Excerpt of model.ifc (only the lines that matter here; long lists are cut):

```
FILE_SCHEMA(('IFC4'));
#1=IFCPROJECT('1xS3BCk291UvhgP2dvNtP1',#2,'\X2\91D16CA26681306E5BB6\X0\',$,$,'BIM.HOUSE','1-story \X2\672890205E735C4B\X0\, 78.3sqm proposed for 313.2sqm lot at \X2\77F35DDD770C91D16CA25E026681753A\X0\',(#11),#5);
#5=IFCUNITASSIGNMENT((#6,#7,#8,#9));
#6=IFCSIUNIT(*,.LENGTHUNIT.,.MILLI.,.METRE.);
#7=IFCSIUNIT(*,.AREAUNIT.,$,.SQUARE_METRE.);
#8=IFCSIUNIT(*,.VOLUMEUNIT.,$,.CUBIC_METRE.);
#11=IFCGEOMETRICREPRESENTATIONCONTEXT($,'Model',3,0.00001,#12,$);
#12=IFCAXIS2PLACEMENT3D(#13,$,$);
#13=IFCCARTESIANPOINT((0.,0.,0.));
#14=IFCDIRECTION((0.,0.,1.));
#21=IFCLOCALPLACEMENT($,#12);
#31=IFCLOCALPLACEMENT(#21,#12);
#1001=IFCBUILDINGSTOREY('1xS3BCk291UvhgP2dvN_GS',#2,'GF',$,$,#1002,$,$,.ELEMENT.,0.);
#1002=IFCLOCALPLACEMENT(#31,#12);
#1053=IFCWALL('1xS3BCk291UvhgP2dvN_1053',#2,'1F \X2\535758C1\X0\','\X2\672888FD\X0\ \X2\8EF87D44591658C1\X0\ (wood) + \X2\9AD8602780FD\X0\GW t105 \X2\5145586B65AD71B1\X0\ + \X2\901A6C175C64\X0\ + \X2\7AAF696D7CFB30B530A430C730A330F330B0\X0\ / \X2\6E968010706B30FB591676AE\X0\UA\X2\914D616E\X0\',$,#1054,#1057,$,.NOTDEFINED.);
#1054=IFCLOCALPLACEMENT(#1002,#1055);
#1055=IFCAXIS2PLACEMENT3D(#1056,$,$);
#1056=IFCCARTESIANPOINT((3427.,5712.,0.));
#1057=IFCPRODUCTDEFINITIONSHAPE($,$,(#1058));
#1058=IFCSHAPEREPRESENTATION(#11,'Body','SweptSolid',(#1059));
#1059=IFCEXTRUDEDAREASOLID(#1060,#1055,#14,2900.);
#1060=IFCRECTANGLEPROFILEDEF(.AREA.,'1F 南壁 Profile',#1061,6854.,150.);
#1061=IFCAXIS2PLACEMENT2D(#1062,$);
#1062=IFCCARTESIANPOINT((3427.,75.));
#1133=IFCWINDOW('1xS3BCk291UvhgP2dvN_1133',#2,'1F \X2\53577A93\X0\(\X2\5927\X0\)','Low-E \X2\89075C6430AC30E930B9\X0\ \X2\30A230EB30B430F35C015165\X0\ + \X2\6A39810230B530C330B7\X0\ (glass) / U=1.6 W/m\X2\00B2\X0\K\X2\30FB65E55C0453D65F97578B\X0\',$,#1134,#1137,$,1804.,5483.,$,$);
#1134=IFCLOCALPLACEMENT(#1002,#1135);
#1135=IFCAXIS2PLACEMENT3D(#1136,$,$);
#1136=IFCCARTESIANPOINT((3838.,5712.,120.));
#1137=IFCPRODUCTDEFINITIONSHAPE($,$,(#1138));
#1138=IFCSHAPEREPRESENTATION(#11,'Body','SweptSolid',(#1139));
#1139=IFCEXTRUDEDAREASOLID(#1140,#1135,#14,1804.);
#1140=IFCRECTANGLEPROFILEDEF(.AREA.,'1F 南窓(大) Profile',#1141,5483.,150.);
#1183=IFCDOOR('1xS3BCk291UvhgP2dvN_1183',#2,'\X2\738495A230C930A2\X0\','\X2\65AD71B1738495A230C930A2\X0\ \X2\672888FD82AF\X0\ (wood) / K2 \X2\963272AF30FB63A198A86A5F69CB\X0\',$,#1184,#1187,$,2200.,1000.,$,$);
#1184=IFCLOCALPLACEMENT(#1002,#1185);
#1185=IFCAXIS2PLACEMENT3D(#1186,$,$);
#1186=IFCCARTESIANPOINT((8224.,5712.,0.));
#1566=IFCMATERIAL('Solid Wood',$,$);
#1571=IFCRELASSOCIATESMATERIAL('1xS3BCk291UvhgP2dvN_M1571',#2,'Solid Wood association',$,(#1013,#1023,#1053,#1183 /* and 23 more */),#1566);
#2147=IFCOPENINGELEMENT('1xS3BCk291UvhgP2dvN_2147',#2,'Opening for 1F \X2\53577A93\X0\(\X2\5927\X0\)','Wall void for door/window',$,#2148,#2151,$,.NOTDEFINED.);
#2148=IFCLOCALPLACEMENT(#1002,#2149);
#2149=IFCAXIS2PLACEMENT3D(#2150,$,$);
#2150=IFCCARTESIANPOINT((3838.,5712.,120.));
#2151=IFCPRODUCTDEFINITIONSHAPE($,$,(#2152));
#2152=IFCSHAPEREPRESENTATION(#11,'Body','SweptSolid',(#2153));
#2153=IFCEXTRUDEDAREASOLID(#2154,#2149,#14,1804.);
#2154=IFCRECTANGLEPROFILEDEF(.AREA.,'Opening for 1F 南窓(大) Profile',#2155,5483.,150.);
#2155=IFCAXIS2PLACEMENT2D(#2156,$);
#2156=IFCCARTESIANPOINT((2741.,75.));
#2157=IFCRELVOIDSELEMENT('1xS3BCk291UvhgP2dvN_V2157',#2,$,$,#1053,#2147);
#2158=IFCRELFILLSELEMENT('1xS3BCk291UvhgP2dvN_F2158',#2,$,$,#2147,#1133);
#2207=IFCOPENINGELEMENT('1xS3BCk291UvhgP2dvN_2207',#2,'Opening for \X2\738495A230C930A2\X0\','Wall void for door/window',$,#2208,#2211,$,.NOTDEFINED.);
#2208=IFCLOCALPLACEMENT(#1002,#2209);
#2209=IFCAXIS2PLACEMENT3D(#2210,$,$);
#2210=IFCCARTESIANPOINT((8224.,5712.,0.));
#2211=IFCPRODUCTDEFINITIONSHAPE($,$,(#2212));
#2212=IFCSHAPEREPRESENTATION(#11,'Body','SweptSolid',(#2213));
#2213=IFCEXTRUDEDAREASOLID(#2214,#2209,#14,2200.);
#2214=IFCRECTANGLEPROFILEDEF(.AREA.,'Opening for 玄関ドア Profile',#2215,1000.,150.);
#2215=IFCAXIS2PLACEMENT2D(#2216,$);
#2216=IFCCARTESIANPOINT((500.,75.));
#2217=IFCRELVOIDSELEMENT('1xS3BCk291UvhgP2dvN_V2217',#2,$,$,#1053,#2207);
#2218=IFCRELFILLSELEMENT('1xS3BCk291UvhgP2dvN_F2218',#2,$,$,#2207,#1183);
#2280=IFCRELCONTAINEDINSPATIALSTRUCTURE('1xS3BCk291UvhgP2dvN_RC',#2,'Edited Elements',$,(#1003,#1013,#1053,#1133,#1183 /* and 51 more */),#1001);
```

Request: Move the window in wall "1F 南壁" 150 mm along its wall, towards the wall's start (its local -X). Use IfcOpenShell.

```python
import ifcopenshell
import ifcopenshell.api.geometry
import ifcopenshell.util.placement
import ifcopenshell.util.unit

model = ifcopenshell.open("model.ifc")
unit_scale = ifcopenshell.util.unit.calculate_unit_scale(model)

window = model.by_guid("1xS3BCk291UvhgP2dvN_1133")
opening = window.FillsVoids[0].RelatingOpeningElement
wall = opening.VoidsElements[0].RelatingBuildingElement

wall_matrix = ifcopenshell.util.placement.get_local_placement(wall.ObjectPlacement)
shift = wall_matrix[:3, 0] * -0.15 / unit_scale
before = ifcopenshell.util.placement.get_local_placement(window.ObjectPlacement)[:3, 3].copy()

# The window is not placed relative to its opening, so move both.
for product in (opening, window):
    matrix = ifcopenshell.util.placement.get_local_placement(product.ObjectPlacement)
    matrix[:3, 3] += shift
    ifcopenshell.api.geometry.edit_object_placement(model, product=product, matrix=matrix, is_si=False)

after = ifcopenshell.util.placement.get_local_placement(window.ObjectPlacement)[:3, 3]
print("window moved by", (after - before).round(3) + 0.0)

model.write("model_v2.ifc")
```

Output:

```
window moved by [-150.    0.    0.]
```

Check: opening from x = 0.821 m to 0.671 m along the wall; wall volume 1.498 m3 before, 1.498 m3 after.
